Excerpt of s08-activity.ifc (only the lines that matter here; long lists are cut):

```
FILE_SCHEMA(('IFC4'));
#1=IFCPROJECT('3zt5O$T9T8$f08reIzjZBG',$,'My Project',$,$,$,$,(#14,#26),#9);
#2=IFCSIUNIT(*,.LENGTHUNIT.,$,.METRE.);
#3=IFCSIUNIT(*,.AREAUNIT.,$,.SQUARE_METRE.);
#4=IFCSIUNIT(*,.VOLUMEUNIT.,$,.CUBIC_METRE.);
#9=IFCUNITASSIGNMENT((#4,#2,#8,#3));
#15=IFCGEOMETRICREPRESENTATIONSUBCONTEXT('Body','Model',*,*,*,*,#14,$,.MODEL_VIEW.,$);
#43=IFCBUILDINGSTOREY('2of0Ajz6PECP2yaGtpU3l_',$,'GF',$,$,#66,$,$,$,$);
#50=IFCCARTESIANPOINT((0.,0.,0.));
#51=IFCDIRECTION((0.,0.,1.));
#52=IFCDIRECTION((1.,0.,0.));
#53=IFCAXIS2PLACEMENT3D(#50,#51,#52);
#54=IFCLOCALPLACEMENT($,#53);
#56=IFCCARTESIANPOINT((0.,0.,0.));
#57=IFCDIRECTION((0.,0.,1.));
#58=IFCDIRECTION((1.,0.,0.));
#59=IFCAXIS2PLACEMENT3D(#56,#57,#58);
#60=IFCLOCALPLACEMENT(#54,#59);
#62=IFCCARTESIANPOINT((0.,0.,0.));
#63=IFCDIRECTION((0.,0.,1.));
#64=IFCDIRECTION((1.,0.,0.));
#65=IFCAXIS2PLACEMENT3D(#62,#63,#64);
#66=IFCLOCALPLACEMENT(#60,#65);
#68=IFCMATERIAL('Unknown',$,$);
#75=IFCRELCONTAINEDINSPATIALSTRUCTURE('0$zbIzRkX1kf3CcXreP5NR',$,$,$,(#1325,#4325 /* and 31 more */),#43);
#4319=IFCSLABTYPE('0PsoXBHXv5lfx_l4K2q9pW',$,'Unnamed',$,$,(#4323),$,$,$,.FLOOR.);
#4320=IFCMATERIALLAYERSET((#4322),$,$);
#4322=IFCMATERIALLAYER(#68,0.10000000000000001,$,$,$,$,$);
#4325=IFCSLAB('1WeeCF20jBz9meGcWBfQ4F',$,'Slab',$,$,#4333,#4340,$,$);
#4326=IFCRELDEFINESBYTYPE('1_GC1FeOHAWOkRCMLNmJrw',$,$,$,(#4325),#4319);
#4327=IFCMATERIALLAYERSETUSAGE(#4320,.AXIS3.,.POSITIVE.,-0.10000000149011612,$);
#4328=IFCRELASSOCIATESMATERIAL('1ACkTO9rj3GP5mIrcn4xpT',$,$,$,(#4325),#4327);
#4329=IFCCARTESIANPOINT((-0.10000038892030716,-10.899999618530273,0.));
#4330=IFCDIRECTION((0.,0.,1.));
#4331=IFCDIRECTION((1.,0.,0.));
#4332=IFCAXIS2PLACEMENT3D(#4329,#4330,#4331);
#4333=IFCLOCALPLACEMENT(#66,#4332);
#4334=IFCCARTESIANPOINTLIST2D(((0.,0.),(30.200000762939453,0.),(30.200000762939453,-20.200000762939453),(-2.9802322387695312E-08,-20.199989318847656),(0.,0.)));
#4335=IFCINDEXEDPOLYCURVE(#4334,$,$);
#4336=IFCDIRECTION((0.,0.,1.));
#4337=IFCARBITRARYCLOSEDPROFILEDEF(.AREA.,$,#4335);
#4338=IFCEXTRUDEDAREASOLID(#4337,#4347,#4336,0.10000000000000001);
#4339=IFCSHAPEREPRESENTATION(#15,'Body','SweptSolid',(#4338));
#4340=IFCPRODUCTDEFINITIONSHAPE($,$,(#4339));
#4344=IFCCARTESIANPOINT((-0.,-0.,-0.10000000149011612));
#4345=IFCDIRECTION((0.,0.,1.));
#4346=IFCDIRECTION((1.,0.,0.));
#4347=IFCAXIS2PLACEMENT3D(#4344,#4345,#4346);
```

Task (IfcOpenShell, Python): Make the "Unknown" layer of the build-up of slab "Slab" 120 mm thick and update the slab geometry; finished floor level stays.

```python
import ifcopenshell
import ifcopenshell.util.element
import ifcopenshell.util.representation

model = ifcopenshell.open("s08-activity.ifc")

layer_set = model.by_id(4320)
layer = next(l for l in layer_set.MaterialLayers if l.Material and l.Material.Name == "Unknown")
change = 0.12 - layer.LayerThickness
layer.LayerThickness += change

# Geometry does not follow the layer set by itself.
slabs = [e for e in ifcopenshell.util.element.get_elements_by_material(model, layer_set) if e.is_a("IfcSlab")]
for slab in sorted(slabs, key=lambda e: e.id()):
    body = ifcopenshell.util.representation.get_representation(slab, "Model", "Body")
    solid = body.Items[0]
    old_depth = solid.Depth
    solid.Depth += change
    # Extruded upwards: lower the start of the extrusion so the top stays.
    x, y, z = solid.Position.Location.Coordinates
    solid.Position.Location = model.createIfcCartesianPoint((x, y, z - change))
    print(slab.id(), f"{old_depth:g} -> {solid.Depth:g}")

# The layers are counted up from the underside, which has moved.
for usage in {ifcopenshell.util.element.get_material(slab) for slab in slabs}:
    usage.OffsetFromReferenceLine -= change

model.write("s08-activity_v2.ifc")
```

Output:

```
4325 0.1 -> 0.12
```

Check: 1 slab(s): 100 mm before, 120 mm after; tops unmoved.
